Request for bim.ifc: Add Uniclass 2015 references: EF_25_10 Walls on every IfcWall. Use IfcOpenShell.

First a look at what the model holds.

```python
import ifcopenshell

model = ifcopenshell.open("bim.ifc")
print(model.schema)
print("classifications:", [c.Name for c in model.by_type("IfcClassification")])
for ifc_class in ("IfcDoor", "IfcRoof", "IfcStair", "IfcWall", "IfcWindow"):
    print(ifc_class, len(model.by_type(ifc_class)))
```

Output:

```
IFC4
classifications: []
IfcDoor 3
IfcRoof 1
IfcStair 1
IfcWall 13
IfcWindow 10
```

```python
import ifcopenshell
import ifcopenshell.api.classification

model = ifcopenshell.open("bim.ifc")

system = ifcopenshell.api.classification.add_classification(model, classification="Uniclass 2015")

codes = {
    "IfcWall": ("EF_25_10", "Walls"),
}
for ifc_class, (code, name) in codes.items():
    products = model.by_type(ifc_class)
    ifcopenshell.api.classification.add_reference(
        model, products=products, classification=system, identification=code, name=name
    )
    print(code, len(products))

model.write("bim-out.ifc")
```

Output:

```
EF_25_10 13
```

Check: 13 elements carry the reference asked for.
